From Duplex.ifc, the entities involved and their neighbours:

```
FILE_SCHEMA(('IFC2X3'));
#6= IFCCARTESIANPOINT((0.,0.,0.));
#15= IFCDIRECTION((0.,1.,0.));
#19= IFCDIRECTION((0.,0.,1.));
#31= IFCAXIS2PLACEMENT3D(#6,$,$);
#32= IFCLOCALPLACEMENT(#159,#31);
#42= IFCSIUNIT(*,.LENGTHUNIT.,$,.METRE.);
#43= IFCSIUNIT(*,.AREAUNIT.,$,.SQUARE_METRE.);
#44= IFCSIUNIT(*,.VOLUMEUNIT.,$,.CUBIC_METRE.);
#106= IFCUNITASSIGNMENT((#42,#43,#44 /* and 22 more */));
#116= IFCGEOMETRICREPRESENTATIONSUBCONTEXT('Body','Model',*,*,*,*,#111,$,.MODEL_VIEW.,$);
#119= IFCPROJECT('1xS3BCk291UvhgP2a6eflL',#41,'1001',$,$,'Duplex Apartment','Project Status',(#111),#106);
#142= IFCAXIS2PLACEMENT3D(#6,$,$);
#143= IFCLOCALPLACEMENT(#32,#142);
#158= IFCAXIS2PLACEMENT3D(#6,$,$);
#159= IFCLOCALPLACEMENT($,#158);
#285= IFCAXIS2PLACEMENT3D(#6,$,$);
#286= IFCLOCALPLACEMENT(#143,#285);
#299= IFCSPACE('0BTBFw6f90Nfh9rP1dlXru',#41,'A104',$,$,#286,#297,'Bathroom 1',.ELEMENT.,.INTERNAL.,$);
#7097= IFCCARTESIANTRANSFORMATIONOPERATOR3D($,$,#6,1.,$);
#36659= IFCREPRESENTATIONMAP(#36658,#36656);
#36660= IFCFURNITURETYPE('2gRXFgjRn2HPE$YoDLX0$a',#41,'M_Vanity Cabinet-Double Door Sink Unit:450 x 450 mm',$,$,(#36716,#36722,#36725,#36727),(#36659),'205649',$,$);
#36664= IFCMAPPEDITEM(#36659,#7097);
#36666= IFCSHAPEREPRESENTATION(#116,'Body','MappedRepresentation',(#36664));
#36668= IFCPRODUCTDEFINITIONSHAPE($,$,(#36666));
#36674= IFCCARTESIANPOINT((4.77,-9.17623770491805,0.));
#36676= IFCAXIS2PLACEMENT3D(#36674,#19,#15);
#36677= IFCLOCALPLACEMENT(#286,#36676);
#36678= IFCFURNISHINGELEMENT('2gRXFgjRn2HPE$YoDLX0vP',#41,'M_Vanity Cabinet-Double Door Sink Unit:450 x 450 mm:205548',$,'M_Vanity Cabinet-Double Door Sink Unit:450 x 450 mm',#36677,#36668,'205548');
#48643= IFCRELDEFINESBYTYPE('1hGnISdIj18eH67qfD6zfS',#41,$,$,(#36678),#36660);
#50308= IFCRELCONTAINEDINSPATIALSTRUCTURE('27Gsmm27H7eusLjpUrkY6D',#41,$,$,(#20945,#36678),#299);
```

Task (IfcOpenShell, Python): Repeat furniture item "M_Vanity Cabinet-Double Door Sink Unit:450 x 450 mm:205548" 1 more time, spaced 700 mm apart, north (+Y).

```python
import numpy as np
import ifcopenshell
import ifcopenshell.api.geometry
import ifcopenshell.api.root
import ifcopenshell.util.element
import ifcopenshell.util.placement
import ifcopenshell.util.unit

model = ifcopenshell.open("Duplex.ifc")
unit_scale = ifcopenshell.util.unit.calculate_unit_scale(model)


def reuse_history(source, copy):
    """copy_class also copies each property set's owner history, people and application; keep the originals."""
    for rel in copy.IsDefinedBy:
        if rel.is_a("IfcRelDefinesByProperties") and (history := rel.RelatingPropertyDefinition.OwnerHistory):
            rel.RelatingPropertyDefinition.OwnerHistory = source.OwnerHistory
            ifcopenshell.util.element.remove_deep2(model, history)


source = model.by_guid("2gRXFgjRn2HPE$YoDLX0vP")
base = ifcopenshell.util.placement.get_local_placement(source.ObjectPlacement)
step = np.array([0.0, 1.0, 0.0]) * 0.7 / unit_scale

for i in range(1, 2):
    copy = ifcopenshell.api.root.copy_class(model, product=source)
    copy.Representation = ifcopenshell.util.element.copy_deep(
        model, source.Representation, exclude=["IfcGeometricRepresentationContext", "IfcRepresentationMap"]
    )
    copy.Name = "M_Vanity Cabinet-Double Door Sink Unit:450 x 450 mm"
    copy.Tag = None
    reuse_history(source, copy)
    matrix = base.copy()
    matrix[:3, 3] += i * step
    print("added at", matrix[:3, 3].round(3) + 0.0)
    ifcopenshell.api.geometry.edit_object_placement(model, product=copy, matrix=matrix, is_si=False)

model.write("Duplex_v2.ifc")
```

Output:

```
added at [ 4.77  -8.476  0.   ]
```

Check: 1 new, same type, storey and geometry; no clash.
